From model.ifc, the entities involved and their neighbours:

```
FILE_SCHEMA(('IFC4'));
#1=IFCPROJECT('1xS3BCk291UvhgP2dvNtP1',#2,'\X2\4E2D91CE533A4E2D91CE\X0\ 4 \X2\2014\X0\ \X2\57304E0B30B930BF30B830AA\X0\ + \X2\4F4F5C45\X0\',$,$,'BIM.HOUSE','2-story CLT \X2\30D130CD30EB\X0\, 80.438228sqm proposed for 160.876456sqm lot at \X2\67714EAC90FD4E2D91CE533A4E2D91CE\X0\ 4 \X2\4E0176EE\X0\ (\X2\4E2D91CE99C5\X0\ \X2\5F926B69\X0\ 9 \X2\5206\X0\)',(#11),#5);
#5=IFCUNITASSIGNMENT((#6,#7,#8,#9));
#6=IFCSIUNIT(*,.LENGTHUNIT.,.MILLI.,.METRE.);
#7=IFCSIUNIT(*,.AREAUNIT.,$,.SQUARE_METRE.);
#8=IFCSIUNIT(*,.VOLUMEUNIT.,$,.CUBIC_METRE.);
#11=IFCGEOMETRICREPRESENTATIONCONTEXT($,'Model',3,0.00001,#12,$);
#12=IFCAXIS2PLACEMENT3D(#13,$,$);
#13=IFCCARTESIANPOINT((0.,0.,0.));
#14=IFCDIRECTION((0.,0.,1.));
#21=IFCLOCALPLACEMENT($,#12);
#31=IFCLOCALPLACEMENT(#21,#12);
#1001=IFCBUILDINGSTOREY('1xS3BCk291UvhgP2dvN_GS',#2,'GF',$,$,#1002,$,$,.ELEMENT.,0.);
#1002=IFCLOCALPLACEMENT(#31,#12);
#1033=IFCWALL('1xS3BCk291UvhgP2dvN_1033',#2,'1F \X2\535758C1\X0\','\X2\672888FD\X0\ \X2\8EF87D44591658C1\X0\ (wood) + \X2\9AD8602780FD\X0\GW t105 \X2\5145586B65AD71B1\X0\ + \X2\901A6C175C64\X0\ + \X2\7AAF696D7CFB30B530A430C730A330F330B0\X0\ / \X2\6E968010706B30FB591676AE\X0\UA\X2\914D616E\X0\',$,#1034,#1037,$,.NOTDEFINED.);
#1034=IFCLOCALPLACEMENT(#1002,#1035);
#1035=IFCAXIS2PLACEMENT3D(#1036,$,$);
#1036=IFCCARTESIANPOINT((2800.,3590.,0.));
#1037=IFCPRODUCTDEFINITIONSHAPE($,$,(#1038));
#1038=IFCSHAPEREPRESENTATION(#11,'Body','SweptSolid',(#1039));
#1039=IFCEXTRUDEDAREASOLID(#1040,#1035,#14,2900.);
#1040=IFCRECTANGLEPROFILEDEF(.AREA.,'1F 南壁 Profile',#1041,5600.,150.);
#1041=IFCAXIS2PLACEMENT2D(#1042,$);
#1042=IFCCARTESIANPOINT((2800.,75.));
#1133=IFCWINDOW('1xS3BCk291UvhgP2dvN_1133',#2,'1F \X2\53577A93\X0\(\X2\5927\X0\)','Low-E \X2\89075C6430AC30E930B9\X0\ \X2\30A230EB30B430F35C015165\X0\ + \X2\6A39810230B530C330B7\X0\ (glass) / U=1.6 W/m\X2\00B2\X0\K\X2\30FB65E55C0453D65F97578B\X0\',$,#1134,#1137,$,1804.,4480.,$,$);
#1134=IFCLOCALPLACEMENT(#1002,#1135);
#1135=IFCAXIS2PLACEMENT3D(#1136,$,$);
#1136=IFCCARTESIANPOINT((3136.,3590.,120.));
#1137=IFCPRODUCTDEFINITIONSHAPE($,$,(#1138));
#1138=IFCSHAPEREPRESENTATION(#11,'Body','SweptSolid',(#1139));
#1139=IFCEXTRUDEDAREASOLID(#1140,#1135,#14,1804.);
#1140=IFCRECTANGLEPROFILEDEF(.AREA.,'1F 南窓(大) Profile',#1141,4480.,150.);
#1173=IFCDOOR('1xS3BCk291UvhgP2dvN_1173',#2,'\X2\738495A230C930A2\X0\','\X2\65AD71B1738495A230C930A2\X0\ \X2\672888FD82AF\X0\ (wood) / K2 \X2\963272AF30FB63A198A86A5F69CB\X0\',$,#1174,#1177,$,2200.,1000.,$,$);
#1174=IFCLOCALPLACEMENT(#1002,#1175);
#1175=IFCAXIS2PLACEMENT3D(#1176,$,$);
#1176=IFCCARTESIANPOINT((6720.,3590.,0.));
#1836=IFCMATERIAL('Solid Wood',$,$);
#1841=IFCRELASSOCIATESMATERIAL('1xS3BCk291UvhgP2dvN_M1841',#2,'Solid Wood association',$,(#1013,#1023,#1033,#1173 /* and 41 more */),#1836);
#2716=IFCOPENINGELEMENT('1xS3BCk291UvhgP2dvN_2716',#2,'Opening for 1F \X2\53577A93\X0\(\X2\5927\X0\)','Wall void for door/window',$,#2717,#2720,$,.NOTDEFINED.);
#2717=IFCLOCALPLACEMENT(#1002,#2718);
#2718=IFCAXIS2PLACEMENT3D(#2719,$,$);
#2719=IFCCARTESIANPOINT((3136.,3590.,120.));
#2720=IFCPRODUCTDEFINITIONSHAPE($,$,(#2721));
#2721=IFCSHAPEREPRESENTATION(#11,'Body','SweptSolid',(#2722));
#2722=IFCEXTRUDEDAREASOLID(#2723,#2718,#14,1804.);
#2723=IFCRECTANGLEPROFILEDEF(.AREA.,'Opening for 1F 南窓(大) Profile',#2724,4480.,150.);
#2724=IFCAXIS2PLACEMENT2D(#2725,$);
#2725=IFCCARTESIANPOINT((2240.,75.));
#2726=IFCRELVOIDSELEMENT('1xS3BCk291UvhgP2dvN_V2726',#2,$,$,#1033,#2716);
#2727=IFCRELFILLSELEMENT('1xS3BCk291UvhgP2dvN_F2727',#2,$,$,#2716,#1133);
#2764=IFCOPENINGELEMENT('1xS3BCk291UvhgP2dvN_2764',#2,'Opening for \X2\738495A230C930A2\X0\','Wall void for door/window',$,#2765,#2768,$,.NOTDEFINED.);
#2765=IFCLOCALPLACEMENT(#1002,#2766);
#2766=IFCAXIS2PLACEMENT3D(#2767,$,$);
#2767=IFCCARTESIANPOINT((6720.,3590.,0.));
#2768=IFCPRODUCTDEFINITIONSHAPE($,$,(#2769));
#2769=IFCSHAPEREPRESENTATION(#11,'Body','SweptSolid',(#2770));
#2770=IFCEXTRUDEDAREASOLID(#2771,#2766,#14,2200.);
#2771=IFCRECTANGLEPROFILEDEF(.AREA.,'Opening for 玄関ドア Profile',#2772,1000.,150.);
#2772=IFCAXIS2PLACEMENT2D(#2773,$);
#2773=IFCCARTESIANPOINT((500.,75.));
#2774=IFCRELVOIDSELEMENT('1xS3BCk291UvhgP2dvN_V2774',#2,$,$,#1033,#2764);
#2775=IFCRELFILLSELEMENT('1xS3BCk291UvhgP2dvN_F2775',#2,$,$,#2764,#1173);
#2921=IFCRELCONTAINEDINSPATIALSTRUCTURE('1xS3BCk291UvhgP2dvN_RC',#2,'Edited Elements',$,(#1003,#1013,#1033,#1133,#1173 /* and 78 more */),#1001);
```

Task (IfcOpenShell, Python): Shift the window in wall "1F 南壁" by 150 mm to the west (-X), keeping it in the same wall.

```python
import ifcopenshell
import ifcopenshell.api.geometry
import ifcopenshell.util.placement

model = ifcopenshell.open("model.ifc")

window = model.by_guid("1xS3BCk291UvhgP2dvN_1133")
opening = window.FillsVoids[0].RelatingOpeningElement
wall = opening.VoidsElements[0].RelatingBuildingElement

wall_matrix = ifcopenshell.util.placement.get_local_placement(wall.ObjectPlacement)
shift = wall_matrix[:3, 0] * -150.0
before = ifcopenshell.util.placement.get_local_placement(window.ObjectPlacement)[:3, 3].copy()

# The window is not placed relative to its opening, so move both.
for product in (opening, window):
    matrix = ifcopenshell.util.placement.get_local_placement(product.ObjectPlacement)
    matrix[:3, 3] += shift
    ifcopenshell.api.geometry.edit_object_placement(model, product=product, matrix=matrix, is_si=False)

after = ifcopenshell.util.placement.get_local_placement(window.ObjectPlacement)[:3, 3]
print("window moved by", (after - before).round(3) + 0.0)

model.write("model_edited.ifc")
```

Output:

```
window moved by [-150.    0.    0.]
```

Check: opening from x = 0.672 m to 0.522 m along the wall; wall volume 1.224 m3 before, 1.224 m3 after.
